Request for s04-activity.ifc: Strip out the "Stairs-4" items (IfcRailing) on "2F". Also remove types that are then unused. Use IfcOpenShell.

First a look at what the model holds.

```python
import ifcopenshell
import ifcopenshell.util.element

model = ifcopenshell.open("s04-activity.ifc")
print(model.schema)
storey = next(s for s in model.by_type("IfcBuildingStorey") if s.Name == "2F")
railings = [e for e in ifcopenshell.util.element.get_decomposition(storey) if e.is_a("IfcRailing")]
seen = {}
for e in railings:
    element_type = ifcopenshell.util.element.get_type(e)
    name = element_type.Name if element_type not in (None, e) else None
    seen[name] = seen.get(name, 0) + 1
for name, count in sorted(seen.items(), key=str):
    print(count, "x", name)
```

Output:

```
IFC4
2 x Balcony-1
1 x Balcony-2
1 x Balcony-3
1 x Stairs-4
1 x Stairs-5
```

```python
import ifcopenshell
import ifcopenshell.api.root
import ifcopenshell.util.element

model = ifcopenshell.open("s04-activity.ifc")

storey = next(s for s in model.by_type("IfcBuildingStorey") if s.Name == "2F")
railings = [e for e in ifcopenshell.util.element.get_decomposition(storey) if e.is_a("IfcRailing")]
targets = [e for e in railings if (t := ifcopenshell.util.element.get_type(e)) not in (None, e) and t.Name == "Stairs-4"]
types = {ifcopenshell.util.element.get_type(e) for e in targets} - {None, *targets}

for e in targets:
    ifcopenshell.api.root.remove_product(model, product=e)
print(len(targets), "removed")

unused = [t for t in types if not ifcopenshell.util.element.get_types(t)]
for t in unused:
    ifcopenshell.api.root.remove_product(model, product=t)
print(len(unused), "unused types removed")

model.write("s04-activity-out.ifc")
```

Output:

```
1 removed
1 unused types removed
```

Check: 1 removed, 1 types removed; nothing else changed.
